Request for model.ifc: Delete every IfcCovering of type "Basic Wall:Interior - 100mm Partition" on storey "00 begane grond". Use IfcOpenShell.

First a look at what the model holds.

```python
import ifcopenshell
import ifcopenshell.util.element

model = ifcopenshell.open("model.ifc")
print(model.schema)
storey = next(s for s in model.by_type("IfcBuildingStorey") if s.Name == "00 begane grond")
coverings = [e for e in ifcopenshell.util.element.get_decomposition(storey) if e.is_a("IfcCovering")]
seen = {}
for e in coverings:
    element_type = ifcopenshell.util.element.get_type(e)
    name = element_type.Name if element_type not in (None, e) else None
    seen[name] = seen.get(name, 0) + 1
for name, count in sorted(seen.items(), key=str):
    print(count, "x", name)
```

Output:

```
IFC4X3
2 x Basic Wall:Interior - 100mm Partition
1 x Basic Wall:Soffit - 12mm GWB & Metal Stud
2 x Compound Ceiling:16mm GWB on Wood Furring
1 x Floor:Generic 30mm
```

```python
import ifcopenshell
import ifcopenshell.api.root
import ifcopenshell.util.element

model = ifcopenshell.open("model.ifc")

storey = next(s for s in model.by_type("IfcBuildingStorey") if s.Name == "00 begane grond")
coverings = [e for e in ifcopenshell.util.element.get_decomposition(storey) if e.is_a("IfcCovering")]
targets = [e for e in coverings if (t := ifcopenshell.util.element.get_type(e)) not in (None, e) and t.Name == "Basic Wall:Interior - 100mm Partition"]

for e in targets:
    ifcopenshell.api.root.remove_product(model, product=e)
print(len(targets), "removed")

model.write("model_updated.ifc")
```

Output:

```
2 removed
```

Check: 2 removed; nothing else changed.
